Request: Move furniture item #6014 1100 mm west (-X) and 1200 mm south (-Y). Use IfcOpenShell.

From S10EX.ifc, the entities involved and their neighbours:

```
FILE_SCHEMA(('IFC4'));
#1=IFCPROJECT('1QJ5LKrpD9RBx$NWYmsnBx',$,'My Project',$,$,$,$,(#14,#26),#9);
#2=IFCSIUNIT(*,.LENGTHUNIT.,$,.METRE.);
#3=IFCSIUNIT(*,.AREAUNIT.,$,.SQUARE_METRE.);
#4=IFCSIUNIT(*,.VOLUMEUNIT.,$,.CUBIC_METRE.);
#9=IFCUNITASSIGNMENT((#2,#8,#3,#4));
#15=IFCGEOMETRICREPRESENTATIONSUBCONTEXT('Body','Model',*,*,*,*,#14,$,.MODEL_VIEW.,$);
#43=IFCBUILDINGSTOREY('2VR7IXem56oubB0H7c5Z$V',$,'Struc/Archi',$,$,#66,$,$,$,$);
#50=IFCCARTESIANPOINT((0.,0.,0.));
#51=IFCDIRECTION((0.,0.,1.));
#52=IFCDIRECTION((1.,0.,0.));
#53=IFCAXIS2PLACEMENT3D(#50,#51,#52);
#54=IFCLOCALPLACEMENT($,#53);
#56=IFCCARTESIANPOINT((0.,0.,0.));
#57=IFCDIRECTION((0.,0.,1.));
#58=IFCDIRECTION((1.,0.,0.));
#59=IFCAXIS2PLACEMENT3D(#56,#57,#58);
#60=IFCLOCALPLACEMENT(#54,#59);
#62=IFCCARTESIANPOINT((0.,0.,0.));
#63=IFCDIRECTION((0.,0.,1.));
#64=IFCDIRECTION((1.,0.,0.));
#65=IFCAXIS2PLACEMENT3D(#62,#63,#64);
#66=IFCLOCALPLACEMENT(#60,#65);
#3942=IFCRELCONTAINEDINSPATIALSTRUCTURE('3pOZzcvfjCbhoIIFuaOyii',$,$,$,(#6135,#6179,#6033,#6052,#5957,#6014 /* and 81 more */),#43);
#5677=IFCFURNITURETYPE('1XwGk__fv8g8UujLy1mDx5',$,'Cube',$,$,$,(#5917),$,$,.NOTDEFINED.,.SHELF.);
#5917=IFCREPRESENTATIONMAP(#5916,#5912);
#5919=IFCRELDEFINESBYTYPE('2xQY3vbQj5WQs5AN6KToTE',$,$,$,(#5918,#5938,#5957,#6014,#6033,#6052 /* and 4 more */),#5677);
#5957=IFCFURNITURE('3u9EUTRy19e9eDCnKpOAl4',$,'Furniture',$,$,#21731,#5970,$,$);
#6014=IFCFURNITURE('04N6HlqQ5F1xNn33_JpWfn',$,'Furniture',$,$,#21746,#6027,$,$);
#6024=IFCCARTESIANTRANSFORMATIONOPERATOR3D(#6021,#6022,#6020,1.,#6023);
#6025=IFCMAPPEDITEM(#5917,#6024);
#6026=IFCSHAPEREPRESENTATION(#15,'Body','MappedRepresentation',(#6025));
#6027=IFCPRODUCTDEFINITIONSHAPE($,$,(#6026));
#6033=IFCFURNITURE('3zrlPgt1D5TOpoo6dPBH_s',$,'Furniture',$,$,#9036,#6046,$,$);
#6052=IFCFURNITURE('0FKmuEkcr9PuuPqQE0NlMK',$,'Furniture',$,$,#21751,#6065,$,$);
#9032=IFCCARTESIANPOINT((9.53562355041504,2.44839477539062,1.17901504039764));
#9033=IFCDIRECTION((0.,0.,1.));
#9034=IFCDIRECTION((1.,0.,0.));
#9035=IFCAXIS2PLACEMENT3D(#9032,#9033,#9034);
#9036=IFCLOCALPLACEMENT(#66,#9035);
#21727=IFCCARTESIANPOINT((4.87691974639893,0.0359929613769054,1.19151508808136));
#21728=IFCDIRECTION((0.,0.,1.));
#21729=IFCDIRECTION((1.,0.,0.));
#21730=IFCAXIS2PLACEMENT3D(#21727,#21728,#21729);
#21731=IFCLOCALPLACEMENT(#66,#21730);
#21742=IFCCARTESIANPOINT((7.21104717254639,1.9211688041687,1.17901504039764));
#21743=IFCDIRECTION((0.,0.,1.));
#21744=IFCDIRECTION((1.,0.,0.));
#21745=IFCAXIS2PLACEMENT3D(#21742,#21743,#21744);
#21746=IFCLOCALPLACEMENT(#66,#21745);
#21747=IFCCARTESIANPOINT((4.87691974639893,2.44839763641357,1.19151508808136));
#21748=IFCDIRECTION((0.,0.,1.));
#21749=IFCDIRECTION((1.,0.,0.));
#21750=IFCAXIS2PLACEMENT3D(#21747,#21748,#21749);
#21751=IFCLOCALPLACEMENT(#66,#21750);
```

```python
import ifcopenshell
import ifcopenshell.api.geometry
import ifcopenshell.util.placement

model = ifcopenshell.open("S10EX.ifc")

item = model.by_id(6014)
matrix = ifcopenshell.util.placement.get_local_placement(item.ObjectPlacement)
matrix[0, 3] -= 1.1
matrix[1, 3] -= 1.2
ifcopenshell.api.geometry.edit_object_placement(model, product=item, matrix=matrix, is_si=False)

print(ifcopenshell.util.placement.get_local_placement(item.ObjectPlacement).round(3) + 0.0)

model.write("S10EX-out.ifc")
```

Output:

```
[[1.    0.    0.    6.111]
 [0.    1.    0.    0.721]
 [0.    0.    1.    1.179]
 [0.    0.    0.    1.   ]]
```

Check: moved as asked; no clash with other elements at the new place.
